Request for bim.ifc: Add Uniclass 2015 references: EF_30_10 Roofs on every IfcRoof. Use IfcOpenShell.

First a look at what the model holds.

```python
import ifcopenshell

model = ifcopenshell.open("bim.ifc")
print(model.schema)
print("classifications:", [c.Name for c in model.by_type("IfcClassification")])
for ifc_class in ("IfcDoor", "IfcRoof", "IfcStair", "IfcWall", "IfcWindow"):
    print(ifc_class, len(model.by_type(ifc_class)))
```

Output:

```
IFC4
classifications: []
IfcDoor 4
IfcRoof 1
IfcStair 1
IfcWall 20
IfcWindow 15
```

```python
import ifcopenshell
import ifcopenshell.api.classification

model = ifcopenshell.open("bim.ifc")

system = ifcopenshell.api.classification.add_classification(model, classification="Uniclass 2015")

codes = {
    "IfcRoof": ("EF_30_10", "Roofs"),
}
for ifc_class, (code, name) in codes.items():
    products = model.by_type(ifc_class)
    ifcopenshell.api.classification.add_reference(
        model, products=products, classification=system, identification=code, name=name
    )
    print(code, len(products))

model.write("bim-out.ifc")
```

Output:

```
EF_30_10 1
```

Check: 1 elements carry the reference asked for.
